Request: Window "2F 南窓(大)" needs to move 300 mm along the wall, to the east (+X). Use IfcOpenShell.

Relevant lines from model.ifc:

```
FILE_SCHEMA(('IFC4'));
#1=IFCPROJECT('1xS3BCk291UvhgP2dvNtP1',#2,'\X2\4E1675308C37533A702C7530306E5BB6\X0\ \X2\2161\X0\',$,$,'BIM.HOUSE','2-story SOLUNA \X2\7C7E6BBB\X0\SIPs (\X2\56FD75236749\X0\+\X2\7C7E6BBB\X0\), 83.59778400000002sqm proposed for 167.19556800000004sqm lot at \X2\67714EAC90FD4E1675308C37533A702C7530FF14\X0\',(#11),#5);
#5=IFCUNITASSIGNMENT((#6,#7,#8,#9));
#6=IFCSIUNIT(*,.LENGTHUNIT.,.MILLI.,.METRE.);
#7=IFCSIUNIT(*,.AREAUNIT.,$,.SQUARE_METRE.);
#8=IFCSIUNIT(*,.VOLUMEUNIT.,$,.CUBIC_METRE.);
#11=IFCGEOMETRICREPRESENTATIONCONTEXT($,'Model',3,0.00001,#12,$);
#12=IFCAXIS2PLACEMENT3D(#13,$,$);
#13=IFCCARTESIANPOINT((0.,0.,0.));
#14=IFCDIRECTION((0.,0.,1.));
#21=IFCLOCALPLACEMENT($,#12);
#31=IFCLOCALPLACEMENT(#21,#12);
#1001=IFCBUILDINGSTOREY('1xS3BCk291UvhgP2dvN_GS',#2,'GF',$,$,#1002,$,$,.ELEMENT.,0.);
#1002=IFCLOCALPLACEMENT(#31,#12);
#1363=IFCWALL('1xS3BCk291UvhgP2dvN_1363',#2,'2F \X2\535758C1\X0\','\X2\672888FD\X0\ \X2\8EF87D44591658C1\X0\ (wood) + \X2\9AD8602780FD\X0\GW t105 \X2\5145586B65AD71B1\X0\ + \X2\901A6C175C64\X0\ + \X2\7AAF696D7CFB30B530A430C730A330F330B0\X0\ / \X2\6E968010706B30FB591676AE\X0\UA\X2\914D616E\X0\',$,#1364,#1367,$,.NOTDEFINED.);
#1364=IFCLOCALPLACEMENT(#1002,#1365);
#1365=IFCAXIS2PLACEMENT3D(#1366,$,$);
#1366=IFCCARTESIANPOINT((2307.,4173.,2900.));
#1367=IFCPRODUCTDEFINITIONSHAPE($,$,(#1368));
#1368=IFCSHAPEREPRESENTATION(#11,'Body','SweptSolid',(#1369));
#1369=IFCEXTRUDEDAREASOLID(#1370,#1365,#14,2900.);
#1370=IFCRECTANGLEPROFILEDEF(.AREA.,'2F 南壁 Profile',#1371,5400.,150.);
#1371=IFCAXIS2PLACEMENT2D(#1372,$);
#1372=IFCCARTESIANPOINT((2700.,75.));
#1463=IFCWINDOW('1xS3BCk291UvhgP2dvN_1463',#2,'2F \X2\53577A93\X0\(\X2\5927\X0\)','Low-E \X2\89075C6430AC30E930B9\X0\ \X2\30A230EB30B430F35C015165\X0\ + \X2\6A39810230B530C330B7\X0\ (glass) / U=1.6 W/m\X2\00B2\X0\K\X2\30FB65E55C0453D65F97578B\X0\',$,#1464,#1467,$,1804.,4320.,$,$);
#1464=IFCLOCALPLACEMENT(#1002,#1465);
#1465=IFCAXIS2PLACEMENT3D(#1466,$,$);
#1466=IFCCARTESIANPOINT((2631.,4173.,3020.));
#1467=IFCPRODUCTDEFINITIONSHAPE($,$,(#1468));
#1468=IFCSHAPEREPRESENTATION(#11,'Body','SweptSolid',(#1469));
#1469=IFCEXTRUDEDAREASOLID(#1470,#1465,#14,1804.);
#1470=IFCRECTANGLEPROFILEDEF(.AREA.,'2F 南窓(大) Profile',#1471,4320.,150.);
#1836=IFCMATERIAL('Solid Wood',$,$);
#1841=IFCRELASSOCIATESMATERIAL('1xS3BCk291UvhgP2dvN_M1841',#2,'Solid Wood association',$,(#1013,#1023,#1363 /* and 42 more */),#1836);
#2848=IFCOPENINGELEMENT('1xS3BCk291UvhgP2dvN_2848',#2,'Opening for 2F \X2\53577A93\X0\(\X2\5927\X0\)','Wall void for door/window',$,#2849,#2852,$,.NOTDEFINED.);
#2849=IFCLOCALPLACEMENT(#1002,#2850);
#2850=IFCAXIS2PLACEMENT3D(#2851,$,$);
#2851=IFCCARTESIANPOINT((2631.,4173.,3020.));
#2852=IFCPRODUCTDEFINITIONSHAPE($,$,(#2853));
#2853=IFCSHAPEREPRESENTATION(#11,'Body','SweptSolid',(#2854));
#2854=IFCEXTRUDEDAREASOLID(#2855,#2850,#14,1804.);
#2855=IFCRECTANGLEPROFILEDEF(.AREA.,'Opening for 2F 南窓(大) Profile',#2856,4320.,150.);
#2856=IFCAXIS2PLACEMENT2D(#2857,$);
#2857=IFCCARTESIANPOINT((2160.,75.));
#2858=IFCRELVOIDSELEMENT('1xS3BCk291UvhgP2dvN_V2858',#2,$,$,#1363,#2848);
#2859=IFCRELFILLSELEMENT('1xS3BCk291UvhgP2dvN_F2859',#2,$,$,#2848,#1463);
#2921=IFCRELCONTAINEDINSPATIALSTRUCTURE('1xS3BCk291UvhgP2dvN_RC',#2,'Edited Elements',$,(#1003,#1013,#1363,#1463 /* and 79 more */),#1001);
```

```python
import ifcopenshell
import ifcopenshell.api.geometry
import ifcopenshell.util.placement
import ifcopenshell.util.unit

model = ifcopenshell.open("model.ifc")
unit_scale = ifcopenshell.util.unit.calculate_unit_scale(model)

window = model.by_id(1463)
opening = window.FillsVoids[0].RelatingOpeningElement
wall = opening.VoidsElements[0].RelatingBuildingElement

wall_matrix = ifcopenshell.util.placement.get_local_placement(wall.ObjectPlacement)
shift = wall_matrix[:3, 0] * 0.3 / unit_scale
before = ifcopenshell.util.placement.get_local_placement(window.ObjectPlacement)[:3, 3].copy()

# The window is not placed relative to its opening, so move both.
for product in (opening, window):
    matrix = ifcopenshell.util.placement.get_local_placement(product.ObjectPlacement)
    matrix[:3, 3] += shift
    ifcopenshell.api.geometry.edit_object_placement(model, product=product, matrix=matrix, is_si=False)

after = ifcopenshell.util.placement.get_local_placement(window.ObjectPlacement)[:3, 3]
print("window moved by", (after - before).round(3) + 0.0)

model.write("model_updated.ifc")
```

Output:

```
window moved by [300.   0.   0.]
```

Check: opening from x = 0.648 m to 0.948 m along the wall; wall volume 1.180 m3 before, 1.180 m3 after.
